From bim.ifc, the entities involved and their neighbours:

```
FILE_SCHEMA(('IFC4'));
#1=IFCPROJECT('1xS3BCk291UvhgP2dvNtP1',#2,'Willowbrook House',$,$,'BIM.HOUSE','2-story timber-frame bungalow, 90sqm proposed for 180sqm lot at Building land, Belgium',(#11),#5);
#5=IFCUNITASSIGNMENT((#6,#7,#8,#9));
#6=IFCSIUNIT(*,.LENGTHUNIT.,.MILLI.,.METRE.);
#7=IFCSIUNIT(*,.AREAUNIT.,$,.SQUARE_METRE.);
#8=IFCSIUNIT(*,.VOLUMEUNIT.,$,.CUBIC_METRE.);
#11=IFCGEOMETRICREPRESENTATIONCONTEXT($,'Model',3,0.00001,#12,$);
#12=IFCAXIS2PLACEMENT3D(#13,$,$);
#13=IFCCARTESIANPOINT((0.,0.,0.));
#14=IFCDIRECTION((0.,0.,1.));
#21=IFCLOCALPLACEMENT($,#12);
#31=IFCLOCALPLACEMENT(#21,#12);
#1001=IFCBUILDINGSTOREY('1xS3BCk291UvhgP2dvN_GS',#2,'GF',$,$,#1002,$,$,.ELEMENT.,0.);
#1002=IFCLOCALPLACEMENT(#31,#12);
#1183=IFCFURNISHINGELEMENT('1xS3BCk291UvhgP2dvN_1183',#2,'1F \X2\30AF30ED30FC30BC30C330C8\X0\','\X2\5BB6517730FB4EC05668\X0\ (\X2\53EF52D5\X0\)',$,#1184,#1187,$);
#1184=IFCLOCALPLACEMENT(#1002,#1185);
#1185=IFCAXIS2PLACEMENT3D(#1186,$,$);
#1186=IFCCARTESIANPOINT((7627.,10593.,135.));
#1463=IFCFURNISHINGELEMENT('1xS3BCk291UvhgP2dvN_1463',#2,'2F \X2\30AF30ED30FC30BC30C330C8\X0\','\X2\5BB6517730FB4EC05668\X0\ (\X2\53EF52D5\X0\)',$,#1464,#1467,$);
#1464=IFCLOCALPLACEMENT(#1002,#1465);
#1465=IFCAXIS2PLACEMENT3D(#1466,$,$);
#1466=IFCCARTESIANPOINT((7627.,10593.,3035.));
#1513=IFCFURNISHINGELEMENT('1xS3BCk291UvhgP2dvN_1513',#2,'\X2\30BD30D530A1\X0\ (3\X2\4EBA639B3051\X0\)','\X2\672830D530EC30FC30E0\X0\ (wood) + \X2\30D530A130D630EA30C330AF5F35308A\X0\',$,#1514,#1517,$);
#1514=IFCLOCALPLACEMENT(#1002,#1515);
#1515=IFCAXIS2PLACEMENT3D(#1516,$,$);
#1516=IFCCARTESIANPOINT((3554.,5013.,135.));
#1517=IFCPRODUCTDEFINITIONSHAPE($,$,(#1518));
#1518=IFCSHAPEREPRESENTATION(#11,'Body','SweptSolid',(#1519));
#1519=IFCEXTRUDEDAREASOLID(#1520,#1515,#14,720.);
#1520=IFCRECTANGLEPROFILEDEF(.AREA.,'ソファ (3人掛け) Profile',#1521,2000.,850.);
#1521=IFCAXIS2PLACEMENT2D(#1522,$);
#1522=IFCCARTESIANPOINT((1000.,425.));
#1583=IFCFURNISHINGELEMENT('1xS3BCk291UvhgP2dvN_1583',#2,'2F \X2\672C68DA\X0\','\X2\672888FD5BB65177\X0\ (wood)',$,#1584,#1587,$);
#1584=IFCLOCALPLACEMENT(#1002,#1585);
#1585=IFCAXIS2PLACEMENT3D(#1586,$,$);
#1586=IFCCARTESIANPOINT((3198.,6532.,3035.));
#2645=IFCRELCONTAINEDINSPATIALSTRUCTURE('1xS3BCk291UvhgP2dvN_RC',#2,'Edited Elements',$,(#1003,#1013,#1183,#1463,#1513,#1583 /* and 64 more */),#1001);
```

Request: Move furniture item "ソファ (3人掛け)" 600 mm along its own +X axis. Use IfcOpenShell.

```python
import ifcopenshell
import ifcopenshell.api.geometry
import ifcopenshell.util.placement

model = ifcopenshell.open("bim.ifc")

item = model.by_guid("1xS3BCk291UvhgP2dvN_1513")
matrix = ifcopenshell.util.placement.get_local_placement(item.ObjectPlacement)
matrix[:3, 3] += matrix[:3, 0] * 600.0
ifcopenshell.api.geometry.edit_object_placement(model, product=item, matrix=matrix, is_si=False)

print(ifcopenshell.util.placement.get_local_placement(item.ObjectPlacement).round(3) + 0.0)

model.write("bim_rev.ifc")
```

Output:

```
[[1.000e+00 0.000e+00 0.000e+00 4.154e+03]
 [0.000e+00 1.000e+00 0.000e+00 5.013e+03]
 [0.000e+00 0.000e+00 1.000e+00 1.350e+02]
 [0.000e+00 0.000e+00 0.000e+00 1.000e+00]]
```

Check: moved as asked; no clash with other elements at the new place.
